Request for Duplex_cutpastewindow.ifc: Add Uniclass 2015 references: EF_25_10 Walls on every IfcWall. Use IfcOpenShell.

First a look at what the model holds.

```python
import ifcopenshell

model = ifcopenshell.open("Duplex_cutpastewindow.ifc")
print(model.schema)
print("classifications:", [c.Name for c in model.by_type("IfcClassification")])
for ifc_class in ("IfcDoor", "IfcRoof", "IfcStair", "IfcWall", "IfcWindow"):
    print(ifc_class, len(model.by_type(ifc_class)))
```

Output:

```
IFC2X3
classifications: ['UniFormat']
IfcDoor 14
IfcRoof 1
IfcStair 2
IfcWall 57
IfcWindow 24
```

```python
import ifcopenshell
import ifcopenshell.api.classification

model = ifcopenshell.open("Duplex_cutpastewindow.ifc")

# IFC2X3 requires Source and Edition and has no link from the project to the system.
system = model.create_entity("IfcClassification", Source="NBS", Edition="2015", Name="Uniclass 2015")

codes = {
    "IfcWall": ("EF_25_10", "Walls"),
}
for ifc_class, (code, name) in codes.items():
    products = model.by_type(ifc_class)
    ifcopenshell.api.classification.add_reference(
        model, products=products, classification=system, identification=code, name=name
    )
    print(code, len(products))

model.write("Duplex_cutpastewindow_rev.ifc")
```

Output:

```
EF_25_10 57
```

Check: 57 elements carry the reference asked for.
